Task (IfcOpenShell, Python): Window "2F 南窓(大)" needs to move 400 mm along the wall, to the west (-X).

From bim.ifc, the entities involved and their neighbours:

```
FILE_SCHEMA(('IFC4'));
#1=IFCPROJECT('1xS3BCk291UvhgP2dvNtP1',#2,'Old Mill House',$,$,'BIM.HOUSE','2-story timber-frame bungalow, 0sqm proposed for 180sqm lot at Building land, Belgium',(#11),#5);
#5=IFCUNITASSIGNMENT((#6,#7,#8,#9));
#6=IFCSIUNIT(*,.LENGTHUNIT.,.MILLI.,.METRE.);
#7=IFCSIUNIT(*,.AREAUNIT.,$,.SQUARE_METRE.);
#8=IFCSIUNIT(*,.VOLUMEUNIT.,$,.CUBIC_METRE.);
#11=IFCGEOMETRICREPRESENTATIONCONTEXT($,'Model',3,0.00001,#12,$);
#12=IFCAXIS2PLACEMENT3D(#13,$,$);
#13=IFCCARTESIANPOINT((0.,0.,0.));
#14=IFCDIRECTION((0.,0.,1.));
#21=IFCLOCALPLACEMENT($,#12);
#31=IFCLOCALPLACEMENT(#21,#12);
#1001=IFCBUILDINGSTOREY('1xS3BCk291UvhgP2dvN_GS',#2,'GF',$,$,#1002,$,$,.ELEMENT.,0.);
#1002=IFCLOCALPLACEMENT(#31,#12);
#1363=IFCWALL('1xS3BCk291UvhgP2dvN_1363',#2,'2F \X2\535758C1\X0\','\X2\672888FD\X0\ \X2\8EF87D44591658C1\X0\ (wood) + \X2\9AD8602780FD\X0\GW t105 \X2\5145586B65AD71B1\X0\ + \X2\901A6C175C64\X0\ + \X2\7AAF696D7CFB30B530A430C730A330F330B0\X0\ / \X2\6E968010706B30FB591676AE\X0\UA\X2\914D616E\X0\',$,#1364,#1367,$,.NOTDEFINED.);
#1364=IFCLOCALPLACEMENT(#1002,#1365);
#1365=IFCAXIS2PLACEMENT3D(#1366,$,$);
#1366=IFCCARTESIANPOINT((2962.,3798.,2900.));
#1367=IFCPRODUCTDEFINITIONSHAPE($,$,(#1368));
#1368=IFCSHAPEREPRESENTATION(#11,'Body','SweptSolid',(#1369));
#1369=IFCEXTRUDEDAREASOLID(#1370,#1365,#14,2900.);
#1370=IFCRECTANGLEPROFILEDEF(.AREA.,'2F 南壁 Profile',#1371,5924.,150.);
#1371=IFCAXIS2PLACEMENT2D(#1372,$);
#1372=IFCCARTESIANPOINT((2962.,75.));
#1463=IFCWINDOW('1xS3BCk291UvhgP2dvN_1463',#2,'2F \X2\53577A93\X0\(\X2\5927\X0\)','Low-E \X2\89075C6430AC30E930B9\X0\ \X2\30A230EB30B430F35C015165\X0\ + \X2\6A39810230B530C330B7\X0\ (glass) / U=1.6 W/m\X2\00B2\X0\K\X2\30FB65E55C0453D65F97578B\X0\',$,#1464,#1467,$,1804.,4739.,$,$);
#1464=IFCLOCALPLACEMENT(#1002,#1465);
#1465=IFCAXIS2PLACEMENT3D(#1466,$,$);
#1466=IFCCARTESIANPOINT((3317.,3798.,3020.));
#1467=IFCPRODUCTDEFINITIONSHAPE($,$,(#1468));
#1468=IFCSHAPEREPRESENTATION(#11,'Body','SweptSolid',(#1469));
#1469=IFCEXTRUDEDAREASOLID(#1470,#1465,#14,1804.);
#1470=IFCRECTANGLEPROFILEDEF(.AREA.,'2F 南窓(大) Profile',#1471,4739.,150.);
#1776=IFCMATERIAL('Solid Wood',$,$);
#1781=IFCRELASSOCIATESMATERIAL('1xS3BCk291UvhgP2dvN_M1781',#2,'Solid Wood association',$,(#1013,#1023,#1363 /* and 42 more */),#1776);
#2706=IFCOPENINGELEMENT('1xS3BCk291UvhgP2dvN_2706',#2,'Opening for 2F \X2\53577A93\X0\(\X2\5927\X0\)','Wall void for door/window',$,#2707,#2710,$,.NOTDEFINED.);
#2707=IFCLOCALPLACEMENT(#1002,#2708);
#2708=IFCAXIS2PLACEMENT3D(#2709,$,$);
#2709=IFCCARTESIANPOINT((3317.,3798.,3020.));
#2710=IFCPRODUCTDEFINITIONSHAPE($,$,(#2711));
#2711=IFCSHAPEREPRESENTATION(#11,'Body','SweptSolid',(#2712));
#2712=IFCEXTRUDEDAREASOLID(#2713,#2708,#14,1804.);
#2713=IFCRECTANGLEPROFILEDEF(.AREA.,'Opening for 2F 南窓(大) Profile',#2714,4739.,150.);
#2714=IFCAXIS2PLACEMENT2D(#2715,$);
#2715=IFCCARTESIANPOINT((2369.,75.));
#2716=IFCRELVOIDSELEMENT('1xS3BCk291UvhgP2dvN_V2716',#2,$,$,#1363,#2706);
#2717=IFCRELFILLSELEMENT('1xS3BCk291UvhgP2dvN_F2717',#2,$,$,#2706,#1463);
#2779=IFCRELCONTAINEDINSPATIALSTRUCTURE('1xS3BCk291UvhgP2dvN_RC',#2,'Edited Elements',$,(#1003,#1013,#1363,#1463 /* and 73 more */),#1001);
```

```python
import ifcopenshell
import ifcopenshell.api.geometry
import ifcopenshell.util.placement
import ifcopenshell.util.unit

model = ifcopenshell.open("bim.ifc")
unit_scale = ifcopenshell.util.unit.calculate_unit_scale(model)

window = model.by_id(1463)
opening = window.FillsVoids[0].RelatingOpeningElement
wall = opening.VoidsElements[0].RelatingBuildingElement

wall_matrix = ifcopenshell.util.placement.get_local_placement(wall.ObjectPlacement)
shift = wall_matrix[:3, 0] * -0.4 / unit_scale
before = ifcopenshell.util.placement.get_local_placement(window.ObjectPlacement)[:3, 3].copy()

# The window is not placed relative to its opening, so move both.
for product in (opening, window):
    matrix = ifcopenshell.util.placement.get_local_placement(product.ObjectPlacement)
    matrix[:3, 3] += shift
    ifcopenshell.api.geometry.edit_object_placement(model, product=product, matrix=matrix, is_si=False)

after = ifcopenshell.util.placement.get_local_placement(window.ObjectPlacement)[:3, 3]
print("window moved by", (after - before).round(3) + 0.0)

model.write("bim_edited.ifc")
```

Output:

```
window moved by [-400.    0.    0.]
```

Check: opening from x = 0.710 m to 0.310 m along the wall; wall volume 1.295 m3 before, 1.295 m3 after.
